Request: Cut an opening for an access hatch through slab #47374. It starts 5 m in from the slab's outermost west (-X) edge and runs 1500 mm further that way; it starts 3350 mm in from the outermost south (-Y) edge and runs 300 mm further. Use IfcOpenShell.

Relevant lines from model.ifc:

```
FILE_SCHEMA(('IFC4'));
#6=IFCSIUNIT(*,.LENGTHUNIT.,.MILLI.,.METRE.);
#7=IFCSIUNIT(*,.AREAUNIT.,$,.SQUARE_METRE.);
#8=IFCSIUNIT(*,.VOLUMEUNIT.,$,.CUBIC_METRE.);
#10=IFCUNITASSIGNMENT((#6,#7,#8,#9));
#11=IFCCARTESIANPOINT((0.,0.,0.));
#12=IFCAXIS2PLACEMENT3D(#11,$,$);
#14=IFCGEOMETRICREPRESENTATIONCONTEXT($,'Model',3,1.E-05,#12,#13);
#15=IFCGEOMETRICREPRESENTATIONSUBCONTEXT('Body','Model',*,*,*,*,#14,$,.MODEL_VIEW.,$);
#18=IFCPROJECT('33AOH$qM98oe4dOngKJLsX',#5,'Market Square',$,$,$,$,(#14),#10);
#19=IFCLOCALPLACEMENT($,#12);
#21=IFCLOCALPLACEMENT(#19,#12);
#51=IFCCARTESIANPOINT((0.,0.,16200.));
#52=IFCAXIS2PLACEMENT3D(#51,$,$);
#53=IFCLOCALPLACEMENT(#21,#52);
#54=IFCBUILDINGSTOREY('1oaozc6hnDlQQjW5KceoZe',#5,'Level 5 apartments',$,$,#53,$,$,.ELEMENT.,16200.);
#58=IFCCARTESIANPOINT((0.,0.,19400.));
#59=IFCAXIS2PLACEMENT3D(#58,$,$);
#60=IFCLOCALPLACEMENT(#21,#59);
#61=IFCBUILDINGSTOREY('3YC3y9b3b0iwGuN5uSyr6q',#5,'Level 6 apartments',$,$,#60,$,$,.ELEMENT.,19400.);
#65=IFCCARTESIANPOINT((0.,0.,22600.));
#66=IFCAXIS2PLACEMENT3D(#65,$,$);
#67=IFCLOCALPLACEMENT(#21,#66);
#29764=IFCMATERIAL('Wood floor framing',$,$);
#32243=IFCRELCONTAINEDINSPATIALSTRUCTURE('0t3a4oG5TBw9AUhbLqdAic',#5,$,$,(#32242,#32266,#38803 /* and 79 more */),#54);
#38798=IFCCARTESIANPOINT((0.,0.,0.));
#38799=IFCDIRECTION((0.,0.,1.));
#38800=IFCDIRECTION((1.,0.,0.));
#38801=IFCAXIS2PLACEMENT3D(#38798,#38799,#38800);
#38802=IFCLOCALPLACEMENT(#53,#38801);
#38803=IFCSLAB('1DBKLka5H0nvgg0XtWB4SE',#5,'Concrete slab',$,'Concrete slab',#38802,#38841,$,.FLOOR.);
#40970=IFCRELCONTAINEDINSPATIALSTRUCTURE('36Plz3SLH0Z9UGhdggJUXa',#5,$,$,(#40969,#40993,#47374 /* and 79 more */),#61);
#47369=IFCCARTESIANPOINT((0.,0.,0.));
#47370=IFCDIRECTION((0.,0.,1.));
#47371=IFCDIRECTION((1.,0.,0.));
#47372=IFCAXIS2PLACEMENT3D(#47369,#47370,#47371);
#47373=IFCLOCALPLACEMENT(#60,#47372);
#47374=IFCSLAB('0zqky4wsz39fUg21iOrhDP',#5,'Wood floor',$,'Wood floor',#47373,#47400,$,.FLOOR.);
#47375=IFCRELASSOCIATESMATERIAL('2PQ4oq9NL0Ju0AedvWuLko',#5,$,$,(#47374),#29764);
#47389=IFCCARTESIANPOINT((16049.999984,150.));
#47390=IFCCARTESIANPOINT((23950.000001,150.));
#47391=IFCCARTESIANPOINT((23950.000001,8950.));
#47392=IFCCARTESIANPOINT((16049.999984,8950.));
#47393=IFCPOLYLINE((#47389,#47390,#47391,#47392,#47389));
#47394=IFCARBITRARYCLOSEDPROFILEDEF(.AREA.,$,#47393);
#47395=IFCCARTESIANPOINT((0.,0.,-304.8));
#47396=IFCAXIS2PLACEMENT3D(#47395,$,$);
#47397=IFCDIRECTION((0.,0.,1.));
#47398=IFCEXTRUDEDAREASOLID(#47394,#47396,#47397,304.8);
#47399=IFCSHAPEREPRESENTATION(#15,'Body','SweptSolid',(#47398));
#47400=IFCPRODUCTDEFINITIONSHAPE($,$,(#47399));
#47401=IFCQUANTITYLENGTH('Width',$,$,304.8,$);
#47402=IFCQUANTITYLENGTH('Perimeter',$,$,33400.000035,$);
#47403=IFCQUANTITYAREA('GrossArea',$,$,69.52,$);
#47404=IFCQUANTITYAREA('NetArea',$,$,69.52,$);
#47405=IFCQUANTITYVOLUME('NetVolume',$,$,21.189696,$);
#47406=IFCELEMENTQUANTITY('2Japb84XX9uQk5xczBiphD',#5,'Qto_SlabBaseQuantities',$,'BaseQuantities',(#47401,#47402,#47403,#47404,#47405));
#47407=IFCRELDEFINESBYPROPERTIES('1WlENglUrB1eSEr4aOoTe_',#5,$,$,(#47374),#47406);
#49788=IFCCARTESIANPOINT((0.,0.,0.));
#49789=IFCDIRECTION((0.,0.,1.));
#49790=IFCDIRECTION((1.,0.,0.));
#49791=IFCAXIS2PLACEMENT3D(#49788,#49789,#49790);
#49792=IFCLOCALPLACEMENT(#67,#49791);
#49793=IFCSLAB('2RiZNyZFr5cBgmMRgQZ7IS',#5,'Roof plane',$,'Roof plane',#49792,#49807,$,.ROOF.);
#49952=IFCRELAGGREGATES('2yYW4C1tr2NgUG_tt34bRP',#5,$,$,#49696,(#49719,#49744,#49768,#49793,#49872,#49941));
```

```python
import numpy as np
import ifcopenshell
import ifcopenshell.api.feature
import ifcopenshell.api.geometry
import ifcopenshell.api.pset
import ifcopenshell.api.root
import ifcopenshell.geom
import ifcopenshell.util.element
import ifcopenshell.util.placement
import ifcopenshell.util.representation
import ifcopenshell.util.shape
import ifcopenshell.util.unit

model = ifcopenshell.open("model.ifc")
unit_scale = ifcopenshell.util.unit.calculate_unit_scale(model)
area_scale = ifcopenshell.util.unit.calculate_unit_scale(model, "AREAUNIT")
volume_scale = ifcopenshell.util.unit.calculate_unit_scale(model, "VOLUMEUNIT")
settings = ifcopenshell.geom.settings()


def volume(element):
    """Net volume in cubic metres, openings subtracted."""
    shape = ifcopenshell.geom.create_shape(settings, element)
    return ifcopenshell.util.shape.get_volume(shape.geometry)


slab = model.by_guid("0zqky4wsz39fUg21iOrhDP")
before = volume(slab)

# Extent in the slab's own axes, in metres. The edges named are its -X and -Y sides.
slab_shape = ifcopenshell.geom.create_shape(settings, slab)
vertices = ifcopenshell.util.shape.get_vertices(slab_shape.geometry)
x_min, y_min, bottom = vertices.min(axis=0)
top = vertices[:, 2].max()

opening = ifcopenshell.api.root.create_entity(model, ifc_class="IfcOpeningElement", name="Access hatch opening", predefined_type="OPENING")
context = ifcopenshell.util.representation.get_context(model, "Model", "Body", "MODEL_VIEW")
width, depth = 1.5, 0.3
outline = [(0.0, 0.0), (width, 0.0), (width, depth), (0.0, depth), (0.0, 0.0)]
# Overshoot both faces by 50 mm so the cut is clean.
shape = ifcopenshell.api.geometry.add_slab_representation(
    model, context=context, depth=top - bottom + 0.1, polyline=outline
)
ifcopenshell.api.geometry.assign_representation(model, product=opening, representation=shape)

matrix = ifcopenshell.util.placement.get_local_placement(slab.ObjectPlacement)
matrix[:, 3] = matrix @ np.append(np.array([x_min + 5, y_min + 3.35, bottom - 0.05]) / unit_scale, 1.0)
ifcopenshell.api.geometry.edit_object_placement(model, product=opening, matrix=matrix, is_si=False)
ifcopenshell.api.feature.add_feature(model, feature=opening, element=slab)

after = volume(slab)

# Update the slab's stored quantities.
qto = model.by_id(ifcopenshell.util.element.get_pset(slab, "Qto_SlabBaseQuantities", should_inherit=False)["id"])
ifcopenshell.api.pset.edit_qto(model, qto=qto, properties={
    "NetArea": after / (top - bottom) / area_scale,
    "NetVolume": after / volume_scale,
})

print(f"slab volume {before:.3f} -> {after:.3f} m3")

model.write("model_rev.ifc")
```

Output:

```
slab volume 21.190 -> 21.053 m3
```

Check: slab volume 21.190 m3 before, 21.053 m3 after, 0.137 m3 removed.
